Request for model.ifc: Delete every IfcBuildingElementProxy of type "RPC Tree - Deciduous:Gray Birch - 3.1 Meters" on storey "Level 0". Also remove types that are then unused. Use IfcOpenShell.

First a look at what the model holds.

```python
import ifcopenshell
import ifcopenshell.util.element

model = ifcopenshell.open("model.ifc")
print(model.schema)
storey = next(s for s in model.by_type("IfcBuildingStorey") if s.Name == "Level 0")
proxies = [e for e in ifcopenshell.util.element.get_decomposition(storey) if e.is_a("IfcBuildingElementProxy")]
seen = {}
for e in proxies:
    element_type = ifcopenshell.util.element.get_type(e)
    name = element_type.Name if element_type not in (None, e) else None
    seen[name] = seen.get(name, 0) + 1
for name, count in sorted(seen.items(), key=str):
    print(count, "x", name)
```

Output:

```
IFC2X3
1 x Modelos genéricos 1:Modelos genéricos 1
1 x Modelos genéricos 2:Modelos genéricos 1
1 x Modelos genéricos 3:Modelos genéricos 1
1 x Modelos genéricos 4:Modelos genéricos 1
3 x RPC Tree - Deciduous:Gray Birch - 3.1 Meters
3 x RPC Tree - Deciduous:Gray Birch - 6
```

```python
import ifcopenshell
import ifcopenshell.api.root
import ifcopenshell.util.element

model = ifcopenshell.open("model.ifc")

storey = next(s for s in model.by_type("IfcBuildingStorey") if s.Name == "Level 0")
proxies = [e for e in ifcopenshell.util.element.get_decomposition(storey) if e.is_a("IfcBuildingElementProxy")]
targets = [e for e in proxies if (t := ifcopenshell.util.element.get_type(e)) not in (None, e) and t.Name == "RPC Tree - Deciduous:Gray Birch - 3.1 Meters"]
types = {ifcopenshell.util.element.get_type(e) for e in targets} - {None, *targets}

for e in targets:
    ifcopenshell.api.root.remove_product(model, product=e)
print(len(targets), "removed")

unused = [t for t in types if not ifcopenshell.util.element.get_types(t)]
for t in unused:
    ifcopenshell.api.root.remove_product(model, product=t)
print(len(unused), "unused types removed")

model.write("model_rev.ifc")
```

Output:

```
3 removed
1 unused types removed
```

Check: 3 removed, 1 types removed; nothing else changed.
